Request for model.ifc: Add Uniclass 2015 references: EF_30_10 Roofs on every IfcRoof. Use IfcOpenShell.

First a look at what the model holds.

```python
import ifcopenshell

model = ifcopenshell.open("model.ifc")
print(model.schema)
print("classifications:", [c.Name for c in model.by_type("IfcClassification")])
for ifc_class in ("IfcDoor", "IfcRoof", "IfcStair", "IfcWall", "IfcWindow"):
    print(ifc_class, len(model.by_type(ifc_class)))
```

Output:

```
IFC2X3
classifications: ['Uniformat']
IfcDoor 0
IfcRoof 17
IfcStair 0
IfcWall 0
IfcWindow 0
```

```python
import ifcopenshell
import ifcopenshell.api.classification

model = ifcopenshell.open("model.ifc")

# IFC2X3 requires Source and Edition and has no link from the project to the system.
system = model.create_entity("IfcClassification", Source="NBS", Edition="2015", Name="Uniclass 2015")

codes = {
    "IfcRoof": ("EF_30_10", "Roofs"),
}
for ifc_class, (code, name) in codes.items():
    products = model.by_type(ifc_class)
    ifcopenshell.api.classification.add_reference(
        model, products=products, classification=system, identification=code, name=name
    )
    print(code, len(products))

model.write("model_updated.ifc")
```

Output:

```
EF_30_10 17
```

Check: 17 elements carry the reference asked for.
